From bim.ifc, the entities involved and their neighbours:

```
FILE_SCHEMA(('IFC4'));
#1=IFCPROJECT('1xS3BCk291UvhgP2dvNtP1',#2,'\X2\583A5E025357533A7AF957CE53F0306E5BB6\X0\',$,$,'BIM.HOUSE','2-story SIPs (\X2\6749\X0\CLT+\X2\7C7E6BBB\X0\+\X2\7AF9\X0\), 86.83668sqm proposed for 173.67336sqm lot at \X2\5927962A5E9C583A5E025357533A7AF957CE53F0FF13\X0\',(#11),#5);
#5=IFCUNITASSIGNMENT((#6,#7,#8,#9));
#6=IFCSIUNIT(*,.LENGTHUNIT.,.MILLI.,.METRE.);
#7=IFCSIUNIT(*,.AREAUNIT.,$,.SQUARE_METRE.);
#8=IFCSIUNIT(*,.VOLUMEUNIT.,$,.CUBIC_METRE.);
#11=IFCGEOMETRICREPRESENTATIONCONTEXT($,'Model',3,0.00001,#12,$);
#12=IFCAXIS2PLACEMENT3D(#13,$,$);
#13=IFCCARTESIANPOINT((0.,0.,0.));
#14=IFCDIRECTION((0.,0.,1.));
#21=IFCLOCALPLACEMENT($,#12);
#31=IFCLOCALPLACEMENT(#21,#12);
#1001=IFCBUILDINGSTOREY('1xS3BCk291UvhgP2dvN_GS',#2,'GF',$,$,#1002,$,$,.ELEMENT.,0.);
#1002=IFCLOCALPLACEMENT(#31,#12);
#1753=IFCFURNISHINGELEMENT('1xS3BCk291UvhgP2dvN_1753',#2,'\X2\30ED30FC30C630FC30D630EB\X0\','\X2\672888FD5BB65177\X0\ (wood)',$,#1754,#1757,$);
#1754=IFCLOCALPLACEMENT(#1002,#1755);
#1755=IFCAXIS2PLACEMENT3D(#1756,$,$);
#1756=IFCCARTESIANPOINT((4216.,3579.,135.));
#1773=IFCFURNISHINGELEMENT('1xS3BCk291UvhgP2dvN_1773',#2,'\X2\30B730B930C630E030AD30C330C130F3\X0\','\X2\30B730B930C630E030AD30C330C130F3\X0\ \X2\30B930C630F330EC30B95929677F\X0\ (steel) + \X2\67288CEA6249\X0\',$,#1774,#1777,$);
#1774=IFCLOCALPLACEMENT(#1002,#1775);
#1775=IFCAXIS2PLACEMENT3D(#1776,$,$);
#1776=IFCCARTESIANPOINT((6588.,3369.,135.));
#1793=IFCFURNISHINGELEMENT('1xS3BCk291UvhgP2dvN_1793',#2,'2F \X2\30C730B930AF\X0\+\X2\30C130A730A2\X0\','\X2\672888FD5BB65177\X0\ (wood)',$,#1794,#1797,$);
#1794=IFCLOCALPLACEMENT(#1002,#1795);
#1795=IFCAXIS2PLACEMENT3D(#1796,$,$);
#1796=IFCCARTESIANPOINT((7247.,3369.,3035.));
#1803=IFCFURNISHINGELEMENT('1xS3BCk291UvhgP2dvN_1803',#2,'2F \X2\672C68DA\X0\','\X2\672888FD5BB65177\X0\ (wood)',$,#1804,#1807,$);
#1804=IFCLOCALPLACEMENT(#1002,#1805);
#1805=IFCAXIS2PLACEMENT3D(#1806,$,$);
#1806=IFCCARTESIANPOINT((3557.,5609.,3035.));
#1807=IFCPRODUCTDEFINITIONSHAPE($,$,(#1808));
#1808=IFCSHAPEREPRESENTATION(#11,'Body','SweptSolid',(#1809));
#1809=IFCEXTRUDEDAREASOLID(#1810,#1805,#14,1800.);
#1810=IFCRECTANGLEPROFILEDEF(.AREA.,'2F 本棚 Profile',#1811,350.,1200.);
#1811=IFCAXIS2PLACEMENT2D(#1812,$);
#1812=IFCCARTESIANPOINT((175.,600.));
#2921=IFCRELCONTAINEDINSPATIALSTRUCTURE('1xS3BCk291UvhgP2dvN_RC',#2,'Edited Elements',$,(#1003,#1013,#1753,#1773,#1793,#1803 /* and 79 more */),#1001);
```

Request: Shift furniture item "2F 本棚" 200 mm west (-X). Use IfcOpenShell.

```python
import ifcopenshell
import ifcopenshell.api.geometry
import ifcopenshell.util.placement

model = ifcopenshell.open("bim.ifc")

item = model.by_guid("1xS3BCk291UvhgP2dvN_1803")
matrix = ifcopenshell.util.placement.get_local_placement(item.ObjectPlacement)
matrix[0, 3] -= 200.0
ifcopenshell.api.geometry.edit_object_placement(model, product=item, matrix=matrix, is_si=False)

print(ifcopenshell.util.placement.get_local_placement(item.ObjectPlacement).round(3) + 0.0)

model.write("bim_updated.ifc")
```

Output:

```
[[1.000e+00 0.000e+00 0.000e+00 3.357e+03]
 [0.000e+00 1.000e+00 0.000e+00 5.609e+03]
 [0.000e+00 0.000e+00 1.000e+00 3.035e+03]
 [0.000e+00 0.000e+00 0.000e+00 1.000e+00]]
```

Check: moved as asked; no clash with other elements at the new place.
